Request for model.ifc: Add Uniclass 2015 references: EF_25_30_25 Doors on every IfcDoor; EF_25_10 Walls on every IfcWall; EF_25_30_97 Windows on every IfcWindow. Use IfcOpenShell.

First a look at what the model holds.

```python
import ifcopenshell

model = ifcopenshell.open("model.ifc")
print(model.schema)
print("classifications:", [c.Name for c in model.by_type("IfcClassification")])
for ifc_class in ("IfcDoor", "IfcRoof", "IfcStair", "IfcWall", "IfcWindow"):
    print(ifc_class, len(model.by_type(ifc_class)))
```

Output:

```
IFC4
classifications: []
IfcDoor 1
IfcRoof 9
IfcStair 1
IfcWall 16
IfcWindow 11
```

```python
import ifcopenshell
import ifcopenshell.api.classification

model = ifcopenshell.open("model.ifc")

system = ifcopenshell.api.classification.add_classification(model, classification="Uniclass 2015")

codes = {
    "IfcDoor": ("EF_25_30_25", "Doors"),
    "IfcWall": ("EF_25_10", "Walls"),
    "IfcWindow": ("EF_25_30_97", "Windows"),
}
for ifc_class, (code, name) in codes.items():
    products = model.by_type(ifc_class)
    ifcopenshell.api.classification.add_reference(
        model, products=products, classification=system, identification=code, name=name
    )
    print(code, len(products))

model.write("model-out.ifc")
```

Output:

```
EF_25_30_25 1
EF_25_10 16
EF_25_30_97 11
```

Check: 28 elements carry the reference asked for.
